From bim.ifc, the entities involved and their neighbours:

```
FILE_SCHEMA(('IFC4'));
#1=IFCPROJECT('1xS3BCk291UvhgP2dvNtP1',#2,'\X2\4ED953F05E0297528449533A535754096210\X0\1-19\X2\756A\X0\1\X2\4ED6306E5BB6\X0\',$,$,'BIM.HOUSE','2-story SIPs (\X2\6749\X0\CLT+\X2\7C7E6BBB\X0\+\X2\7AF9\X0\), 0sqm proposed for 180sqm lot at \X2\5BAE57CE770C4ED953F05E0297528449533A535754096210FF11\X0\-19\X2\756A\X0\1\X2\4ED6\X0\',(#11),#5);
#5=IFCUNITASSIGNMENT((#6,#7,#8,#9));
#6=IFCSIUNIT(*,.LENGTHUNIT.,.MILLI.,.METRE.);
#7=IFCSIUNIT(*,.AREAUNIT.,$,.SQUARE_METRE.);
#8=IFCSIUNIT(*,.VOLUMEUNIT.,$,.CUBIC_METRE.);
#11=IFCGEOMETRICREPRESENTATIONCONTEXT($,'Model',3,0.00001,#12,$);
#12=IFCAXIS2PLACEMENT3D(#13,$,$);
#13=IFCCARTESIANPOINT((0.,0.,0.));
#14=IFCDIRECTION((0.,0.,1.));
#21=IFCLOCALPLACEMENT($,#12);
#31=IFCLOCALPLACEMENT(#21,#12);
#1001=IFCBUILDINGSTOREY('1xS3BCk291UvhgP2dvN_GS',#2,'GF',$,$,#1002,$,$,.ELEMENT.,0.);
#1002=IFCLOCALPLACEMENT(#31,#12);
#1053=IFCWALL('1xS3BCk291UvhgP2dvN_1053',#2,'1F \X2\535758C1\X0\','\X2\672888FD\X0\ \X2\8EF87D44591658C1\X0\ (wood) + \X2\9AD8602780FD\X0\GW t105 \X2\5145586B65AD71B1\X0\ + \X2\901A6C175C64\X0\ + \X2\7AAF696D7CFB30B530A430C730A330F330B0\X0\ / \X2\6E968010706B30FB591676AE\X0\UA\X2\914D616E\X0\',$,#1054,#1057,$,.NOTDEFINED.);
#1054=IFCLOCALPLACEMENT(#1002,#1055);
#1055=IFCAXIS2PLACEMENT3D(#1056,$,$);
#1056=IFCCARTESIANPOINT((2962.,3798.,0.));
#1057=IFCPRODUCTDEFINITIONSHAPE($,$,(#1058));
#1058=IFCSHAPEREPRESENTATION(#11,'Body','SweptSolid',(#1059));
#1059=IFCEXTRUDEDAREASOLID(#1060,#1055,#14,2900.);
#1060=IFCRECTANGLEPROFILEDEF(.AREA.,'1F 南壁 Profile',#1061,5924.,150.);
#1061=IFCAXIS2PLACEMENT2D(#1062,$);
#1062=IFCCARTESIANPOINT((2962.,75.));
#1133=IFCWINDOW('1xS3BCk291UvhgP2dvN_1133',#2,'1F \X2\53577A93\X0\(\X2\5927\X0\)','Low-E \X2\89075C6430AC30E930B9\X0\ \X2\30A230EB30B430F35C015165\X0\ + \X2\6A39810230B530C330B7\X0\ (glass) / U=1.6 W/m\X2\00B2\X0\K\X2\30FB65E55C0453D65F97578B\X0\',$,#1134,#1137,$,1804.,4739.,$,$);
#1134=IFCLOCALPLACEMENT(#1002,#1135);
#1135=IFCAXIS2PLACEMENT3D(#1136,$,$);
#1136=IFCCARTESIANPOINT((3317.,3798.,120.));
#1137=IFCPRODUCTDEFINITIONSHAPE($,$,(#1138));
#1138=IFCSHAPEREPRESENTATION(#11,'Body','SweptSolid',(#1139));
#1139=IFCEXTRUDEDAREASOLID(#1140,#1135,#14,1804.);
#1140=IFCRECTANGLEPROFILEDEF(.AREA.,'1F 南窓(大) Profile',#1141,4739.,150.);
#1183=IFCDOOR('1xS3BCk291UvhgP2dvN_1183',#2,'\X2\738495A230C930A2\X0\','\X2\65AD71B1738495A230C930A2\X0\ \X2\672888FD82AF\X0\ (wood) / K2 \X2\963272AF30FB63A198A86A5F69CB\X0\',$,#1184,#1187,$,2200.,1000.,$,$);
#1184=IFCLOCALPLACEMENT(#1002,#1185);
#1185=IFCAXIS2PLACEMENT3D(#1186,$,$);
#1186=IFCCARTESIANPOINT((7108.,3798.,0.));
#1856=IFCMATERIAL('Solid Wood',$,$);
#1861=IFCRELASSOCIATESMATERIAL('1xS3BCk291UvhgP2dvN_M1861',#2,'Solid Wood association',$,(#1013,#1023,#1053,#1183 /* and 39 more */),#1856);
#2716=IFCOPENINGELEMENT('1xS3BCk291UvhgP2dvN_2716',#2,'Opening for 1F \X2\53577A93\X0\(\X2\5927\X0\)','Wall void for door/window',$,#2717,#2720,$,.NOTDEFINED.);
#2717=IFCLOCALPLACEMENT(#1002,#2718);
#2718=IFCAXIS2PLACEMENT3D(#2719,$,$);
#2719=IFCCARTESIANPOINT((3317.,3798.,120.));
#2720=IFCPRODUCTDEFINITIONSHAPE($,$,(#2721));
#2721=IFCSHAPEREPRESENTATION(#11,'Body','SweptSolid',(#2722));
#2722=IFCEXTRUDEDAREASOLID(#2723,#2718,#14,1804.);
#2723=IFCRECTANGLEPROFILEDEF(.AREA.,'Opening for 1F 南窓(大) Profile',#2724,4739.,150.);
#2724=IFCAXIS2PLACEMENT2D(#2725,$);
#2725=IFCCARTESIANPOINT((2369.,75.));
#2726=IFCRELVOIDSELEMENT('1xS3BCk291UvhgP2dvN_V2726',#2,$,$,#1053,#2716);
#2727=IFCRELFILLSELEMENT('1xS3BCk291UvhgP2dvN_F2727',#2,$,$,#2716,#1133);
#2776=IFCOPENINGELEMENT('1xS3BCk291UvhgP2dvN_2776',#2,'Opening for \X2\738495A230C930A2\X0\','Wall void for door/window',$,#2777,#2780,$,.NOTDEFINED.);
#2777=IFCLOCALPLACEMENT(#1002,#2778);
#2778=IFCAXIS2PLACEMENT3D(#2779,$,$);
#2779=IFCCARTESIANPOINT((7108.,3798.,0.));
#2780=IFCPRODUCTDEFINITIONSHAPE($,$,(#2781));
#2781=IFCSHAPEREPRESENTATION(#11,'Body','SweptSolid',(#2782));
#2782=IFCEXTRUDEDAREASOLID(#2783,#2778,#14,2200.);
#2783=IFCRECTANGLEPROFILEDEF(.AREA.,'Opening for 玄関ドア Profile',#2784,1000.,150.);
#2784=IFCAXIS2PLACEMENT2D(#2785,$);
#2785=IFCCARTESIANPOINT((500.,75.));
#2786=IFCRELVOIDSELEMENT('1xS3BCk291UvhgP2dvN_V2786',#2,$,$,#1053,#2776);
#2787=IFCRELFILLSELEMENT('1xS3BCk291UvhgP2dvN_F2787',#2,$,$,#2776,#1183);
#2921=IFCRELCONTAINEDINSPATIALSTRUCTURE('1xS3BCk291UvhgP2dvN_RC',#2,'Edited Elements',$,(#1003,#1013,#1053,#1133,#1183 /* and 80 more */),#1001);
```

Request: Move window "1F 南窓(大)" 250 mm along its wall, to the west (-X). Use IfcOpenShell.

```python
import ifcopenshell
import ifcopenshell.api.geometry
import ifcopenshell.util.placement
import ifcopenshell.util.unit

model = ifcopenshell.open("bim.ifc")
unit_scale = ifcopenshell.util.unit.calculate_unit_scale(model)

window = model.by_id(1133)
opening = window.FillsVoids[0].RelatingOpeningElement
wall = opening.VoidsElements[0].RelatingBuildingElement

wall_matrix = ifcopenshell.util.placement.get_local_placement(wall.ObjectPlacement)
shift = wall_matrix[:3, 0] * -0.25 / unit_scale
before = ifcopenshell.util.placement.get_local_placement(window.ObjectPlacement)[:3, 3].copy()

# The window is not placed relative to its opening, so move both.
for product in (opening, window):
    matrix = ifcopenshell.util.placement.get_local_placement(product.ObjectPlacement)
    matrix[:3, 3] += shift
    ifcopenshell.api.geometry.edit_object_placement(model, product=product, matrix=matrix, is_si=False)

after = ifcopenshell.util.placement.get_local_placement(window.ObjectPlacement)[:3, 3]
print("window moved by", (after - before).round(3) + 0.0)

model.write("bim_edited.ifc")
```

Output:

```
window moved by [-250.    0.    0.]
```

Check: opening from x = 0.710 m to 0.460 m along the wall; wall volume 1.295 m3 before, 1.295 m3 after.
